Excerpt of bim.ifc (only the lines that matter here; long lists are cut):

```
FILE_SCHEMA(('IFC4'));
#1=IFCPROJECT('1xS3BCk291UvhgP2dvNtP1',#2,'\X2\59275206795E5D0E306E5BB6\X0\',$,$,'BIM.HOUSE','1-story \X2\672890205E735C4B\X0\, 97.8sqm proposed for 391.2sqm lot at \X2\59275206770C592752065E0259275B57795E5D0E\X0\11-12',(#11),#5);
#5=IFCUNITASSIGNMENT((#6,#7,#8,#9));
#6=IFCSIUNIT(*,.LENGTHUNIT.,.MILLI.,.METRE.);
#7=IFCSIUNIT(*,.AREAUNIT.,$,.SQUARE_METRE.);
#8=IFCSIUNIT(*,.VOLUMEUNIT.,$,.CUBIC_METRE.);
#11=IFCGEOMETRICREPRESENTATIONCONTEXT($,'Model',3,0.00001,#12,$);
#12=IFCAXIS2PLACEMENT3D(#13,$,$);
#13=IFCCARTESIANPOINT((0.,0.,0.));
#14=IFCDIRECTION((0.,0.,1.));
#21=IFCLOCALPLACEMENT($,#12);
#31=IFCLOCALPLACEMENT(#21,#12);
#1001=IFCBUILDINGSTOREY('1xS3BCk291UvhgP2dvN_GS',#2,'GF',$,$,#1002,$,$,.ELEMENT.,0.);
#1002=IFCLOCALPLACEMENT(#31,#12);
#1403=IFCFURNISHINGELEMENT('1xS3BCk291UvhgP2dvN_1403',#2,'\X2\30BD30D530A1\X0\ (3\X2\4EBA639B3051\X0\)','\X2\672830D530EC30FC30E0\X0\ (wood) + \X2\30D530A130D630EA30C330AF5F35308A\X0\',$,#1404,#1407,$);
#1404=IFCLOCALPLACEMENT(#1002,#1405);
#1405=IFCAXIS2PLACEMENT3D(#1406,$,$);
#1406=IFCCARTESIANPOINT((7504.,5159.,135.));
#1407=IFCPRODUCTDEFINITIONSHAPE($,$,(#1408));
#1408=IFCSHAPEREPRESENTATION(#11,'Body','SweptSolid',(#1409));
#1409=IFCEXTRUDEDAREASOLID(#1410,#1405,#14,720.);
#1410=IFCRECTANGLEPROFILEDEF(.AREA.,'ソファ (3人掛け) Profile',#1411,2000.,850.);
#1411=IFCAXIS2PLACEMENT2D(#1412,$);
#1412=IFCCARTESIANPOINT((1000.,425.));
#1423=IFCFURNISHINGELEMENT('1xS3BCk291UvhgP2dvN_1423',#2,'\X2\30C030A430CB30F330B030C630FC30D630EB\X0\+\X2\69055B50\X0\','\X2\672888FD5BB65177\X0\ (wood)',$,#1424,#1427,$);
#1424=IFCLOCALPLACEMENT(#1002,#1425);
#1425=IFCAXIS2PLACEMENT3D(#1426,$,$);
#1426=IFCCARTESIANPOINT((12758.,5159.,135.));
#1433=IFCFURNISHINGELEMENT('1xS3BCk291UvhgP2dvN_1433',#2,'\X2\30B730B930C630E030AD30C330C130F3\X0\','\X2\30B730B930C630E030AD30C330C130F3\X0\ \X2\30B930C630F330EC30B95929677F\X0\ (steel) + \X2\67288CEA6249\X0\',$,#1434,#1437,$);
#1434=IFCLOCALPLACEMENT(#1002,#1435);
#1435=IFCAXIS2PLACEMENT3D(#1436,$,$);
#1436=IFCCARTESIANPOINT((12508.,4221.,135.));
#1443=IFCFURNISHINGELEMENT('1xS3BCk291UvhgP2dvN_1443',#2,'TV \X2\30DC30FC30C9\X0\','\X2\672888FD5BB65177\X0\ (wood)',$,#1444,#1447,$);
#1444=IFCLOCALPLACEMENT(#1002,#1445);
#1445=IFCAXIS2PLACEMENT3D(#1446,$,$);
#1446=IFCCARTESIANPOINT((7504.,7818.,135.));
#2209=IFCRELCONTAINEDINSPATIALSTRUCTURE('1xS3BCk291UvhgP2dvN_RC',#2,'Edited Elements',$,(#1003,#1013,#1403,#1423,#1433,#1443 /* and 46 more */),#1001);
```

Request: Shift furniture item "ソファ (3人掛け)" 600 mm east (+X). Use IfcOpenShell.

```python
import ifcopenshell
import ifcopenshell.api.geometry
import ifcopenshell.util.placement
import ifcopenshell.util.unit

model = ifcopenshell.open("bim.ifc")
unit_scale = ifcopenshell.util.unit.calculate_unit_scale(model)

item = model.by_id(1403)
matrix = ifcopenshell.util.placement.get_local_placement(item.ObjectPlacement)
matrix[0, 3] += 0.6 / unit_scale
ifcopenshell.api.geometry.edit_object_placement(model, product=item, matrix=matrix, is_si=False)

print(ifcopenshell.util.placement.get_local_placement(item.ObjectPlacement).round(3) + 0.0)

model.write("bim_v2.ifc")
```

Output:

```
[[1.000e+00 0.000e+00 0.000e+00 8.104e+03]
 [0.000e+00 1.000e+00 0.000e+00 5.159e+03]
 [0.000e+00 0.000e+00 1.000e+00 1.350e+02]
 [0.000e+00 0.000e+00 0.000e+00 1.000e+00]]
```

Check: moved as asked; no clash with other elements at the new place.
